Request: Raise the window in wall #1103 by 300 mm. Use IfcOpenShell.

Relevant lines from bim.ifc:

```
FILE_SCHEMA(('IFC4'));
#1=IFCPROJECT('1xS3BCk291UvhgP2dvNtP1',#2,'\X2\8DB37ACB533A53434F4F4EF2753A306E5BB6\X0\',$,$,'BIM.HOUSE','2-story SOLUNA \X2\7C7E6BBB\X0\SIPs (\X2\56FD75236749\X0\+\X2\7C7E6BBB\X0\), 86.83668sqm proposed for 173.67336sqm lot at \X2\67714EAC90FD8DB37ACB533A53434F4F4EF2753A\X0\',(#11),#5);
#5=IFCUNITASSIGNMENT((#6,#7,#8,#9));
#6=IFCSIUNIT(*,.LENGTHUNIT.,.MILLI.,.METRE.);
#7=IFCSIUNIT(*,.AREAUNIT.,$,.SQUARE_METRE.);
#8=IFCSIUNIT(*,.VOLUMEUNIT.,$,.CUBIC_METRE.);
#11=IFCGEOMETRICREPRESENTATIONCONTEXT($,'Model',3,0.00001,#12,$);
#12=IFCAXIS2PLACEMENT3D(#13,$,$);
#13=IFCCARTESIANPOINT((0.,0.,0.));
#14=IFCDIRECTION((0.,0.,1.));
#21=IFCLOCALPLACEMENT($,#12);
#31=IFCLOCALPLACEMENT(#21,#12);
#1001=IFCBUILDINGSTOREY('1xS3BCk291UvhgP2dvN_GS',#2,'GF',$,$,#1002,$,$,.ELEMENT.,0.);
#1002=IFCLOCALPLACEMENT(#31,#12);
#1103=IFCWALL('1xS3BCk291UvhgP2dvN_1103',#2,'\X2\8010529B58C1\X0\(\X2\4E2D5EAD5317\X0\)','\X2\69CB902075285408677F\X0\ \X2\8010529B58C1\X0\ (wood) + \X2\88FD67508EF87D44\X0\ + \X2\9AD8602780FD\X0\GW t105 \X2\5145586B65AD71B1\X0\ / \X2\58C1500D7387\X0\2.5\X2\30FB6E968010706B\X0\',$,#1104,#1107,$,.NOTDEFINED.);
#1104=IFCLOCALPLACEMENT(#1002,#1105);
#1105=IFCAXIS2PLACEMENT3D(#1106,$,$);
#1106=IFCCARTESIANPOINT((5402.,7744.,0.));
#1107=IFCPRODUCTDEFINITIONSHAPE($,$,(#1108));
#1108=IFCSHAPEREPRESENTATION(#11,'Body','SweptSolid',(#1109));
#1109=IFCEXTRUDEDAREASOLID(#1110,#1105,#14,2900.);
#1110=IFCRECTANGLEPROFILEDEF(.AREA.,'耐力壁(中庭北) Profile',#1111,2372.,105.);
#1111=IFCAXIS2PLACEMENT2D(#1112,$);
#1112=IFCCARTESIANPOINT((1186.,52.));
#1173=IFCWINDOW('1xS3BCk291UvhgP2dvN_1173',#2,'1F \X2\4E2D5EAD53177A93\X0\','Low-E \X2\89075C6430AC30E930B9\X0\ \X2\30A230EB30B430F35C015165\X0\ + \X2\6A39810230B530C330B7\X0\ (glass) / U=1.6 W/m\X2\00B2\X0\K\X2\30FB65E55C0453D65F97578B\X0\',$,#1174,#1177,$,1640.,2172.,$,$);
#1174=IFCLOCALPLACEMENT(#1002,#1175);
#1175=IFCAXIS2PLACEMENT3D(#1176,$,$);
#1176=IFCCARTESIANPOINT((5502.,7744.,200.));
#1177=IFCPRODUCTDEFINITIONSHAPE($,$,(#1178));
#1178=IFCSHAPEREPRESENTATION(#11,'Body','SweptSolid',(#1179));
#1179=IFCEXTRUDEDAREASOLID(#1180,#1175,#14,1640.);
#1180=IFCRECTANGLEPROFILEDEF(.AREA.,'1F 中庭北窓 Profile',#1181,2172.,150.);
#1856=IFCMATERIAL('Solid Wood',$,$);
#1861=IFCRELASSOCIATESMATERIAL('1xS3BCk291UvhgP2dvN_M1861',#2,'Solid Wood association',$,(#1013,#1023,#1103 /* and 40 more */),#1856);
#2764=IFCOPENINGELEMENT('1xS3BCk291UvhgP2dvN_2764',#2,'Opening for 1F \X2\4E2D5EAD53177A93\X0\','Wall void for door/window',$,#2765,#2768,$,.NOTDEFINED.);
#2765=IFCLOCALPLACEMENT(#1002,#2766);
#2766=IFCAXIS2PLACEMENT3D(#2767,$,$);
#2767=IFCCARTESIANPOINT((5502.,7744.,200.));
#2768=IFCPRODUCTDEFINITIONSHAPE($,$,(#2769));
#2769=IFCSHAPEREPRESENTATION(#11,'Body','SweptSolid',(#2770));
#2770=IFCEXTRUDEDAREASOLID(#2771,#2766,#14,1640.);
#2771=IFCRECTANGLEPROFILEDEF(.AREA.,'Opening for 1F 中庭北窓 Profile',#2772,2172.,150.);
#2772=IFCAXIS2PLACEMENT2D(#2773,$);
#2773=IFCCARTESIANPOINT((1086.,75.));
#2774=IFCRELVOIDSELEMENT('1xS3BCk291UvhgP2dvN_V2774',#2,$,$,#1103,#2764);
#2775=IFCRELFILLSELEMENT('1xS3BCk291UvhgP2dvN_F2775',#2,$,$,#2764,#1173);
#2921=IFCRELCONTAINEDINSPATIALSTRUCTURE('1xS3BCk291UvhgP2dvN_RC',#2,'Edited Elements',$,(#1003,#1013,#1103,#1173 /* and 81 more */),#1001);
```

```python
import numpy as np
import ifcopenshell
import ifcopenshell.api.geometry
import ifcopenshell.util.placement
import ifcopenshell.util.unit

model = ifcopenshell.open("bim.ifc")
unit_scale = ifcopenshell.util.unit.calculate_unit_scale(model)

window = model.by_guid("1xS3BCk291UvhgP2dvN_1173")
opening = window.FillsVoids[0].RelatingOpeningElement
dz = 300.0

shift = np.array([0.0, 0.0, dz])
# The window is not placed relative to its opening, so move both.
for product in (opening, window):
    matrix = ifcopenshell.util.placement.get_local_placement(product.ObjectPlacement)
    matrix[:3, 3] += shift
    ifcopenshell.api.geometry.edit_object_placement(model, product=product, matrix=matrix, is_si=False)

print(f"moved by {dz * unit_scale:+.3f} m")

model.write("bim_edited.ifc")
```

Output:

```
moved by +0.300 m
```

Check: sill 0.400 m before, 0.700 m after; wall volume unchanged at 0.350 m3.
